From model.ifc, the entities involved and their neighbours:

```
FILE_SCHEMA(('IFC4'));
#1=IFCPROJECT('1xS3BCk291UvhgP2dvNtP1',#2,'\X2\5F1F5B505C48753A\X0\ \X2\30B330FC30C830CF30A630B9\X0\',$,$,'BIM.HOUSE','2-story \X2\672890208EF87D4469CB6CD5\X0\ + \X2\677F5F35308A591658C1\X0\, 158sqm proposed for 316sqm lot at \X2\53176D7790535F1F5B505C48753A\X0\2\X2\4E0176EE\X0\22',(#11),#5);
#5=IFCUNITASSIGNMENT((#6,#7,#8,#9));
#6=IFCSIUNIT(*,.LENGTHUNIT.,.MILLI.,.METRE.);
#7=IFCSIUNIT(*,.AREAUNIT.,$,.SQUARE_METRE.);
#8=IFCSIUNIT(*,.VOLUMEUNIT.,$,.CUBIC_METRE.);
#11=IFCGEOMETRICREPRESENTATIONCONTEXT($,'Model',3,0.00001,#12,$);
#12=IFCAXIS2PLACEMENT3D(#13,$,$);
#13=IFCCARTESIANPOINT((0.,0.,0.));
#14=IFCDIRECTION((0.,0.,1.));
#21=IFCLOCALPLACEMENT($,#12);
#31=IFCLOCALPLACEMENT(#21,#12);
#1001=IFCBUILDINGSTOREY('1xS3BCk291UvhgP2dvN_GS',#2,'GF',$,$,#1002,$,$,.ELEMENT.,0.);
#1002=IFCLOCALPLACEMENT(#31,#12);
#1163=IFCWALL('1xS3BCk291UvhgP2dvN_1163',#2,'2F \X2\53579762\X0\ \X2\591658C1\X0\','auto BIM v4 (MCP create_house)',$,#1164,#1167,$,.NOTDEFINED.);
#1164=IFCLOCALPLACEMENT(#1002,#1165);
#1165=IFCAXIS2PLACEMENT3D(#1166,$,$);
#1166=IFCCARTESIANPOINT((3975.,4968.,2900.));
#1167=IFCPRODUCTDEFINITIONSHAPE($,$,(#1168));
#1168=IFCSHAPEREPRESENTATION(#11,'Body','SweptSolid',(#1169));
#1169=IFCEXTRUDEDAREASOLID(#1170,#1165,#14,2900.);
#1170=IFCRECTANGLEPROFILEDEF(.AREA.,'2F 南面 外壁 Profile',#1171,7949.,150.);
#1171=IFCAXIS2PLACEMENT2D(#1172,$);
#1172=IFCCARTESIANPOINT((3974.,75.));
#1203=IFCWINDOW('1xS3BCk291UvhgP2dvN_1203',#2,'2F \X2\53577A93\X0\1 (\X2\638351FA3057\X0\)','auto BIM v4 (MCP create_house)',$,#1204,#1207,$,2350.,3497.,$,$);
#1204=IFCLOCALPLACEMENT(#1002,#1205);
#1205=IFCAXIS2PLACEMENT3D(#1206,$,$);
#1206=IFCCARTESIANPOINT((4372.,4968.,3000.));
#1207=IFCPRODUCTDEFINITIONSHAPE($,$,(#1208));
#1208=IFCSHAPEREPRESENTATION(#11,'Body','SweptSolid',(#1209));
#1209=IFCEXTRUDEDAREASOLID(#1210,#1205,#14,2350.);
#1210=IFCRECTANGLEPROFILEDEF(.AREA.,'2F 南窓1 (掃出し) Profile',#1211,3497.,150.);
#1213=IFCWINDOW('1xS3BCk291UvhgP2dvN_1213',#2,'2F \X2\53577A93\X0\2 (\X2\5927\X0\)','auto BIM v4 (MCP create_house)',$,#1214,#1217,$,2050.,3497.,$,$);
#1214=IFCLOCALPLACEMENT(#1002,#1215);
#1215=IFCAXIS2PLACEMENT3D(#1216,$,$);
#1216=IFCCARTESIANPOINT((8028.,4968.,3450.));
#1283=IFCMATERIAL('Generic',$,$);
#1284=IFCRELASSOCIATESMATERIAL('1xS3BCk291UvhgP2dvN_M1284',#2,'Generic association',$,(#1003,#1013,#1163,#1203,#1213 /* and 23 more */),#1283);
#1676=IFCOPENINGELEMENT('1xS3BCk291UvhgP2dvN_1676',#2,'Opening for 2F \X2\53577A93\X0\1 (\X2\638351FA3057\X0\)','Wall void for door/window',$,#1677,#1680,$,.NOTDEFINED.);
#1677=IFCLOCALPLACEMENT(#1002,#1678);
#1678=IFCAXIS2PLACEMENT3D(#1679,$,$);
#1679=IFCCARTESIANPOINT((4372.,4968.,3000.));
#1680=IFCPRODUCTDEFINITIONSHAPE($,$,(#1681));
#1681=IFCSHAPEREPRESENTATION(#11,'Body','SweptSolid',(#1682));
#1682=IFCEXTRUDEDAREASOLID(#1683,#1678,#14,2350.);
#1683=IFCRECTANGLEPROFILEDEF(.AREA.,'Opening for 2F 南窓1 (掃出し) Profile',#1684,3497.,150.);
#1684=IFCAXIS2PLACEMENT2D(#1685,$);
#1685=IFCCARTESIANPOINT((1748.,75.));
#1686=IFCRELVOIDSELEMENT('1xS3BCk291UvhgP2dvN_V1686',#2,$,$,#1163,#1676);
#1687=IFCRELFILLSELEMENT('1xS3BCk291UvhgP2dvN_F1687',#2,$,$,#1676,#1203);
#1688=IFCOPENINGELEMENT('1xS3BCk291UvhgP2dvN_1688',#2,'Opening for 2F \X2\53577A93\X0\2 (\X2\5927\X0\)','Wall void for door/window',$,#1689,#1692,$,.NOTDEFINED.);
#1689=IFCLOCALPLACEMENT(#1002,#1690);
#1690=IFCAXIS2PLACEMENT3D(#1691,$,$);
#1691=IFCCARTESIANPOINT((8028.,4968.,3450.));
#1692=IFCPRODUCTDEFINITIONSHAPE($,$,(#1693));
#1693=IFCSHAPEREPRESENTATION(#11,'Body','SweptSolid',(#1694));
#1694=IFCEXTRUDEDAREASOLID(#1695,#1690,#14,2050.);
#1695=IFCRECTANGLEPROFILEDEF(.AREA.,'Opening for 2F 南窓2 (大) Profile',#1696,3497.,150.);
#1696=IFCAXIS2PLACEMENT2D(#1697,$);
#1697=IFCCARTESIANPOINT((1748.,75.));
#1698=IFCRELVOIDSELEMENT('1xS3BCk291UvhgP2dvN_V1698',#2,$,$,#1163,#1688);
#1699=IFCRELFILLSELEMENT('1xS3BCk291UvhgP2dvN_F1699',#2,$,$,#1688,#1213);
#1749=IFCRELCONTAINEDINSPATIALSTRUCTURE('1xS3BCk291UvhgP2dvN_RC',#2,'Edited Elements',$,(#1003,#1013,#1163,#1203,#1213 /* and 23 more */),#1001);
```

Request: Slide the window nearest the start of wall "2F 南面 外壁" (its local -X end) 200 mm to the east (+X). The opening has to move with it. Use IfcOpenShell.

```python
import ifcopenshell
import ifcopenshell.api.geometry
import ifcopenshell.util.placement
import ifcopenshell.util.unit

model = ifcopenshell.open("model.ifc")
unit_scale = ifcopenshell.util.unit.calculate_unit_scale(model)

window = model.by_id(1203)
opening = window.FillsVoids[0].RelatingOpeningElement
wall = opening.VoidsElements[0].RelatingBuildingElement

wall_matrix = ifcopenshell.util.placement.get_local_placement(wall.ObjectPlacement)
shift = wall_matrix[:3, 0] * 0.2 / unit_scale
before = ifcopenshell.util.placement.get_local_placement(window.ObjectPlacement)[:3, 3].copy()

# The window is not placed relative to its opening, so move both.
for product in (opening, window):
    matrix = ifcopenshell.util.placement.get_local_placement(product.ObjectPlacement)
    matrix[:3, 3] += shift
    ifcopenshell.api.geometry.edit_object_placement(model, product=product, matrix=matrix, is_si=False)

after = ifcopenshell.util.placement.get_local_placement(window.ObjectPlacement)[:3, 3]
print("window moved by", (after - before).round(3) + 0.0)

model.write("model-out.ifc")
```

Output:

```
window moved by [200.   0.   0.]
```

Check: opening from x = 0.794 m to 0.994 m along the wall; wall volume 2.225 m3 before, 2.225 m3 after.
